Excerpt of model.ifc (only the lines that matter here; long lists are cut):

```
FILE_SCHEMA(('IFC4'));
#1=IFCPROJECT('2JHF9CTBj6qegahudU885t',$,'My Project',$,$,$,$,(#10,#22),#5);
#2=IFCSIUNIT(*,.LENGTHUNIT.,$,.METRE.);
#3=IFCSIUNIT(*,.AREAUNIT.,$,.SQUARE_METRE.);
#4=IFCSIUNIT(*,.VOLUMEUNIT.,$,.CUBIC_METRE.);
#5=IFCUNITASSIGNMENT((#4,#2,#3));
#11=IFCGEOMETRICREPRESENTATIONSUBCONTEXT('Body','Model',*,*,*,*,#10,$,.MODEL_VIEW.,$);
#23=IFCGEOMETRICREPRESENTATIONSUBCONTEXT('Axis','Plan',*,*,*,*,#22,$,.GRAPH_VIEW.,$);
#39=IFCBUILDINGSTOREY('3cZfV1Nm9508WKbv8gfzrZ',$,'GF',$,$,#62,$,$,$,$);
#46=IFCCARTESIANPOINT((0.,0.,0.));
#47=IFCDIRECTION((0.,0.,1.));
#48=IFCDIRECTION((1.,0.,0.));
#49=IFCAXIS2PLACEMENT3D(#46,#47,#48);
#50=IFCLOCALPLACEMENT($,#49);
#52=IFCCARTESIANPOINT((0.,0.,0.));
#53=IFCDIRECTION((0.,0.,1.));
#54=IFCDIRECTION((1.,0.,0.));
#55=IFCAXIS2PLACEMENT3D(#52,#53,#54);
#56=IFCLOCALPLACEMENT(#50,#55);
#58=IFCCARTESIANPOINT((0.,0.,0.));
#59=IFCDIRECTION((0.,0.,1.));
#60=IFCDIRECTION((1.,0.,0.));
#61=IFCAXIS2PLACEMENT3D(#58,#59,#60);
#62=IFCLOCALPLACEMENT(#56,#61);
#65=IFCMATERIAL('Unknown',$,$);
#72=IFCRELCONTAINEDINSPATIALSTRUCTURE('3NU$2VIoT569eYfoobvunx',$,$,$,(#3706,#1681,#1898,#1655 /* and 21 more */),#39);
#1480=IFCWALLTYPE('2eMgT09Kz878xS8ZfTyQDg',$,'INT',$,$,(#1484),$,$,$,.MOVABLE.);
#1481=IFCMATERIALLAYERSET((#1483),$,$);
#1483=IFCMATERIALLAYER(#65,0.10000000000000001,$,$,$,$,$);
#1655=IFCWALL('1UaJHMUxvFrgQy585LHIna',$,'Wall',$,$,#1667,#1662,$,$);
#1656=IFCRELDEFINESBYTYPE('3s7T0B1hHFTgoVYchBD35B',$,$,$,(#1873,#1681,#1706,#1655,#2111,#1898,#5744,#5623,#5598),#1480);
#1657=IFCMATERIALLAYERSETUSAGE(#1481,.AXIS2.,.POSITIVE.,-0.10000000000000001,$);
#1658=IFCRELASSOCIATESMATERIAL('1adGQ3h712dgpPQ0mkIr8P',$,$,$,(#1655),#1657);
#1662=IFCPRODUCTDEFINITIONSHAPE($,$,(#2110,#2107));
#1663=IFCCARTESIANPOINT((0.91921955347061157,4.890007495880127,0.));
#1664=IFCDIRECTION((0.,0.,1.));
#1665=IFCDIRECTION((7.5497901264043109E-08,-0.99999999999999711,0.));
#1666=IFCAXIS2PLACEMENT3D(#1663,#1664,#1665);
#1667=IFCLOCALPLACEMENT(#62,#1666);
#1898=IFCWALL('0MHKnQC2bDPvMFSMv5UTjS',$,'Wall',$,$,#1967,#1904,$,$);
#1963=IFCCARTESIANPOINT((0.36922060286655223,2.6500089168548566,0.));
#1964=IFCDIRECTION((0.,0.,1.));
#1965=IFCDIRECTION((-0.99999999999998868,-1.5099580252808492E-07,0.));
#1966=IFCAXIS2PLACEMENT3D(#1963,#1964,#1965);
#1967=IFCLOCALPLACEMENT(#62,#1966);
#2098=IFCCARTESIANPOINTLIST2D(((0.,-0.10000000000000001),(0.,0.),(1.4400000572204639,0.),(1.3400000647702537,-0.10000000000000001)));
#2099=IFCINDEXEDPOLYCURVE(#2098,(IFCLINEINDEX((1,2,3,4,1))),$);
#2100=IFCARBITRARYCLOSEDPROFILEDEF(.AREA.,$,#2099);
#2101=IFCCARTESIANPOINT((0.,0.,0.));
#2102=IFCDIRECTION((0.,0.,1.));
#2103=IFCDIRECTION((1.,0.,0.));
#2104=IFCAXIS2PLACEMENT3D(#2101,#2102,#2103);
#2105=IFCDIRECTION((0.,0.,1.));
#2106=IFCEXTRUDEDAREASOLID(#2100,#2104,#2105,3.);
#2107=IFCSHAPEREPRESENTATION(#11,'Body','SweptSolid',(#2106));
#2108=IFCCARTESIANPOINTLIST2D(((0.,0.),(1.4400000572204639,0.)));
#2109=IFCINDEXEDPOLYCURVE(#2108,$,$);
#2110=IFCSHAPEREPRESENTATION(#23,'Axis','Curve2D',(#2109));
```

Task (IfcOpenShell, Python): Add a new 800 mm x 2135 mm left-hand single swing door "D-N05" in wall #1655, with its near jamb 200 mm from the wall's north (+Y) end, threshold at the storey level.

```python
import numpy as np
import ifcopenshell
import ifcopenshell.api.feature
import ifcopenshell.api.geometry
import ifcopenshell.api.root
import ifcopenshell.api.spatial
import ifcopenshell.geom
import ifcopenshell.util.element
import ifcopenshell.util.placement
import ifcopenshell.util.representation
import ifcopenshell.util.shape
import ifcopenshell.util.unit

model = ifcopenshell.open("model.ifc")
unit_scale = ifcopenshell.util.unit.calculate_unit_scale(model)
settings = ifcopenshell.geom.settings()


def volume(element):
    """Net volume in cubic metres, openings subtracted."""
    shape = ifcopenshell.geom.create_shape(settings, element)
    return ifcopenshell.util.shape.get_volume(shape.geometry)


wall = model.by_guid("1UaJHMUxvFrgQy585LHIna")
storey = ifcopenshell.util.element.get_container(wall, ifc_class="IfcBuildingStorey")
context = ifcopenshell.util.representation.get_context(model, "Model", "Body", "MODEL_VIEW")
before = volume(wall)

width, height, from_end, sill = 0.8, 2.135, 0.2, 0.0  # metres

# The wall runs along its own X axis, and the end named is its -X end.
wall_shape = ifcopenshell.geom.create_shape(settings, wall)
x, y, z = ifcopenshell.util.shape.get_vertices(wall_shape.geometry).T
start = x.min() + from_end
face, thickness = float(y.min()), float(y.max() - y.min())
wall_matrix = ifcopenshell.util.placement.get_local_placement(wall.ObjectPlacement)
level = ifcopenshell.util.placement.get_local_placement(storey.ObjectPlacement)[2, 3]


def in_wall(x, y):
    """Placement at x, y metres in the wall's axes, at sill height."""
    matrix = wall_matrix.copy()
    matrix[:, 3] = wall_matrix @ np.array([x / unit_scale, y / unit_scale, 0.0, 1.0])
    matrix[2, 3] = level + sill / unit_scale
    return matrix


# Opening: a box that overshoots both wall faces by 50 mm.
opening = ifcopenshell.api.root.create_entity(model, ifc_class="IfcOpeningElement", predefined_type="OPENING")
box = ifcopenshell.api.geometry.add_wall_representation(
    model, context=context, length=width, height=height, thickness=thickness + 0.1
)
ifcopenshell.api.geometry.assign_representation(model, product=opening, representation=box)
ifcopenshell.api.geometry.edit_object_placement(model, product=opening, matrix=in_wall(start, face - 0.05), is_si=False)
ifcopenshell.api.feature.add_feature(model, feature=opening, element=wall)

door = ifcopenshell.api.root.create_entity(model, ifc_class="IfcDoor", name="D-N05", predefined_type="DOOR")
door.OverallWidth, door.OverallHeight = width / unit_scale, height / unit_scale
door.OperationType = "SINGLE_SWING_LEFT"
body = ifcopenshell.api.geometry.add_door_representation(
    model,
    context=context,
    overall_width=door.OverallWidth,
    overall_height=door.OverallHeight,
    operation_type="SINGLE_SWING_LEFT",
    lining_properties={"LiningDepth": thickness / unit_scale, "ThresholdDepth": thickness / unit_scale},
)
ifcopenshell.api.geometry.assign_representation(model, product=door, representation=body)
ifcopenshell.api.spatial.assign_container(model, products=[door], relating_structure=storey)
ifcopenshell.api.feature.add_filling(model, opening=opening, element=door)

# The lining spans the wall, so the door starts at the wall face.
ifcopenshell.api.geometry.edit_object_placement(model, product=door, matrix=in_wall(start, face), is_si=False)

after = volume(wall)

print(f"wall volume {before:.3f} -> {after:.3f} m3")

model.write("model_edited.ifc")
```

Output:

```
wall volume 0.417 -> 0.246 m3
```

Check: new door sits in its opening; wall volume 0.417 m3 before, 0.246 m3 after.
